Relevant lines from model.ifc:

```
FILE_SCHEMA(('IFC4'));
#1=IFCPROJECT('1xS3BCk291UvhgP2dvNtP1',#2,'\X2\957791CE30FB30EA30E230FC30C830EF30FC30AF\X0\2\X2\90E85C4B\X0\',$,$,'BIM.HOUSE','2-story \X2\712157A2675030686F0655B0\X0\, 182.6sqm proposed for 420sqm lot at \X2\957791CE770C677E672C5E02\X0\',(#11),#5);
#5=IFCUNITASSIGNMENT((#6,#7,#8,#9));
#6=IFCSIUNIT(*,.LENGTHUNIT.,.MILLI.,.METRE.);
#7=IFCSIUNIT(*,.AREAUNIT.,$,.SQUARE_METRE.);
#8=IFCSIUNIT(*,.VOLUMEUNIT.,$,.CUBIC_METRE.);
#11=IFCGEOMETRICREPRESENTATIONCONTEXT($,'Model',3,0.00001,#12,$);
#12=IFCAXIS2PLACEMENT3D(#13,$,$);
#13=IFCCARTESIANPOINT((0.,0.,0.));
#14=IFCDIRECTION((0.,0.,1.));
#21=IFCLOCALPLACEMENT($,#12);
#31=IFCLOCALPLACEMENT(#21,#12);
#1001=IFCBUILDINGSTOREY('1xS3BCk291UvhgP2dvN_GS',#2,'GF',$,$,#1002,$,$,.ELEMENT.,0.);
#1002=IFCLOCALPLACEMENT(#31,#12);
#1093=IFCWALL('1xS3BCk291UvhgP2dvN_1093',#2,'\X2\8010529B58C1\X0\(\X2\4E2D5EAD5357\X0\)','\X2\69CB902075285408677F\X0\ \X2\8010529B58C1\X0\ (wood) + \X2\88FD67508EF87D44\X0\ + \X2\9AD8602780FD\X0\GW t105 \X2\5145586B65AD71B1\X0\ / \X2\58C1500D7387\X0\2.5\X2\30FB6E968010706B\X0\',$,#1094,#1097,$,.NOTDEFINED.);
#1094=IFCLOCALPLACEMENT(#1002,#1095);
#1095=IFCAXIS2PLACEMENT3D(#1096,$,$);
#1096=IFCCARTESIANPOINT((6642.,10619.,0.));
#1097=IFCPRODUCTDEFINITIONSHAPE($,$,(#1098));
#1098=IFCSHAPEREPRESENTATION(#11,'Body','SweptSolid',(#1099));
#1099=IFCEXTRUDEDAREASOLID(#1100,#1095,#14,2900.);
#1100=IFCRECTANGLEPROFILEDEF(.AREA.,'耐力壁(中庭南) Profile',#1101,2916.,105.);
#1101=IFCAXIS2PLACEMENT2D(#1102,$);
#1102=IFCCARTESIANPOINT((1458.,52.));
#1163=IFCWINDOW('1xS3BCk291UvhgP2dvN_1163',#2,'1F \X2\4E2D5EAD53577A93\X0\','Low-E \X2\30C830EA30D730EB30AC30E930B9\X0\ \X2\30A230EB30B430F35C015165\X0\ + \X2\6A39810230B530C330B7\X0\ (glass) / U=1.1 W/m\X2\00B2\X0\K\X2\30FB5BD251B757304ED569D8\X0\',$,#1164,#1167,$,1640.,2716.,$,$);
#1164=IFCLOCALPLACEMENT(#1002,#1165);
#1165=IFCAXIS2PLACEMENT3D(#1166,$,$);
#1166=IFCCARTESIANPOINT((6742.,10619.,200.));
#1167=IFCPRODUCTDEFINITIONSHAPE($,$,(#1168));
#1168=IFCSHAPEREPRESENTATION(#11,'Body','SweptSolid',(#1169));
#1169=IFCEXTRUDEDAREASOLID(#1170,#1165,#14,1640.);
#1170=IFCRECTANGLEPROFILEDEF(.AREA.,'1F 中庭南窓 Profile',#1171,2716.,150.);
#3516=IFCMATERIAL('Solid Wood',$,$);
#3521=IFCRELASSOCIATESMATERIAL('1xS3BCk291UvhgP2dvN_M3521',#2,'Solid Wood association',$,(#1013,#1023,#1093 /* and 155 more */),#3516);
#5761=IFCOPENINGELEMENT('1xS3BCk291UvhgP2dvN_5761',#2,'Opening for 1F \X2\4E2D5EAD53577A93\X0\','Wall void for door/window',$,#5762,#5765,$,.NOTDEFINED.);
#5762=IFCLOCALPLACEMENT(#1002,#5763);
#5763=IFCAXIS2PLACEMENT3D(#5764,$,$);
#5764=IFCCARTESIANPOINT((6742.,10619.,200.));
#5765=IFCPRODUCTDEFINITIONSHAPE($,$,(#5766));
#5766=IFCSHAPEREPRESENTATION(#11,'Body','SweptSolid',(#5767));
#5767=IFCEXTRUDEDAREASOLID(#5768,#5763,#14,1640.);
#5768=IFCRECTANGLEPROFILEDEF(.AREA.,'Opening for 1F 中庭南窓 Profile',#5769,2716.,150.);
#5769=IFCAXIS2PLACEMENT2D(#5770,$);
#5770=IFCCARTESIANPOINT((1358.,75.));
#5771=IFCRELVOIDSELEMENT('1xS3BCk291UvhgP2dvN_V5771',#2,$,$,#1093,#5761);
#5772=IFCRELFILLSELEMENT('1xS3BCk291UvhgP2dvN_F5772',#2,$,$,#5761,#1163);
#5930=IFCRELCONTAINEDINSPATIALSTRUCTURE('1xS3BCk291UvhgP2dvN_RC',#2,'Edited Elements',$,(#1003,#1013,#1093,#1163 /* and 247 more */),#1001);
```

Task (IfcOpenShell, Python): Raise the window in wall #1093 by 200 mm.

```python
import numpy as np
import ifcopenshell
import ifcopenshell.api.geometry
import ifcopenshell.util.placement
import ifcopenshell.util.unit

model = ifcopenshell.open("model.ifc")
unit_scale = ifcopenshell.util.unit.calculate_unit_scale(model)

window = model.by_guid("1xS3BCk291UvhgP2dvN_1163")
opening = window.FillsVoids[0].RelatingOpeningElement
dz = 0.2 / unit_scale

shift = np.array([0.0, 0.0, dz])
# The window is not placed relative to its opening, so move both.
for product in (opening, window):
    matrix = ifcopenshell.util.placement.get_local_placement(product.ObjectPlacement)
    matrix[:3, 3] += shift
    ifcopenshell.api.geometry.edit_object_placement(model, product=product, matrix=matrix, is_si=False)

print(f"moved by {dz * unit_scale:+.3f} m")

model.write("model_updated.ifc")
```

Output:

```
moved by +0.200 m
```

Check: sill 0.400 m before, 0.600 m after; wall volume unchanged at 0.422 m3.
